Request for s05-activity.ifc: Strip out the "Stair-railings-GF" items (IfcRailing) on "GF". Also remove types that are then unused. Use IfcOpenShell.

First a look at what the model holds.

```python
import ifcopenshell
import ifcopenshell.util.element

model = ifcopenshell.open("s05-activity.ifc")
print(model.schema)
storey = next(s for s in model.by_type("IfcBuildingStorey") if s.Name == "GF")
railings = [e for e in ifcopenshell.util.element.get_decomposition(storey) if e.is_a("IfcRailing")]
seen = {}
for e in railings:
    element_type = ifcopenshell.util.element.get_type(e)
    name = element_type.Name if element_type not in (None, e) else None
    seen[name] = seen.get(name, 0) + 1
for name, count in sorted(seen.items(), key=str):
    print(count, "x", name)
```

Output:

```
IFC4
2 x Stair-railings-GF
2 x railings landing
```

```python
import ifcopenshell
import ifcopenshell.api.root
import ifcopenshell.util.element

model = ifcopenshell.open("s05-activity.ifc")

storey = next(s for s in model.by_type("IfcBuildingStorey") if s.Name == "GF")
railings = [e for e in ifcopenshell.util.element.get_decomposition(storey) if e.is_a("IfcRailing")]
targets = [e for e in railings if (t := ifcopenshell.util.element.get_type(e)) not in (None, e) and t.Name == "Stair-railings-GF"]
types = {ifcopenshell.util.element.get_type(e) for e in targets} - {None, *targets}

for e in targets:
    ifcopenshell.api.root.remove_product(model, product=e)
print(len(targets), "removed")

unused = [t for t in types if not ifcopenshell.util.element.get_types(t)]
for t in unused:
    ifcopenshell.api.root.remove_product(model, product=t)
print(len(unused), "unused types removed")

model.write("s05-activity_edited.ifc")
```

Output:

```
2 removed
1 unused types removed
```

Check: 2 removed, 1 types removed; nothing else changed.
